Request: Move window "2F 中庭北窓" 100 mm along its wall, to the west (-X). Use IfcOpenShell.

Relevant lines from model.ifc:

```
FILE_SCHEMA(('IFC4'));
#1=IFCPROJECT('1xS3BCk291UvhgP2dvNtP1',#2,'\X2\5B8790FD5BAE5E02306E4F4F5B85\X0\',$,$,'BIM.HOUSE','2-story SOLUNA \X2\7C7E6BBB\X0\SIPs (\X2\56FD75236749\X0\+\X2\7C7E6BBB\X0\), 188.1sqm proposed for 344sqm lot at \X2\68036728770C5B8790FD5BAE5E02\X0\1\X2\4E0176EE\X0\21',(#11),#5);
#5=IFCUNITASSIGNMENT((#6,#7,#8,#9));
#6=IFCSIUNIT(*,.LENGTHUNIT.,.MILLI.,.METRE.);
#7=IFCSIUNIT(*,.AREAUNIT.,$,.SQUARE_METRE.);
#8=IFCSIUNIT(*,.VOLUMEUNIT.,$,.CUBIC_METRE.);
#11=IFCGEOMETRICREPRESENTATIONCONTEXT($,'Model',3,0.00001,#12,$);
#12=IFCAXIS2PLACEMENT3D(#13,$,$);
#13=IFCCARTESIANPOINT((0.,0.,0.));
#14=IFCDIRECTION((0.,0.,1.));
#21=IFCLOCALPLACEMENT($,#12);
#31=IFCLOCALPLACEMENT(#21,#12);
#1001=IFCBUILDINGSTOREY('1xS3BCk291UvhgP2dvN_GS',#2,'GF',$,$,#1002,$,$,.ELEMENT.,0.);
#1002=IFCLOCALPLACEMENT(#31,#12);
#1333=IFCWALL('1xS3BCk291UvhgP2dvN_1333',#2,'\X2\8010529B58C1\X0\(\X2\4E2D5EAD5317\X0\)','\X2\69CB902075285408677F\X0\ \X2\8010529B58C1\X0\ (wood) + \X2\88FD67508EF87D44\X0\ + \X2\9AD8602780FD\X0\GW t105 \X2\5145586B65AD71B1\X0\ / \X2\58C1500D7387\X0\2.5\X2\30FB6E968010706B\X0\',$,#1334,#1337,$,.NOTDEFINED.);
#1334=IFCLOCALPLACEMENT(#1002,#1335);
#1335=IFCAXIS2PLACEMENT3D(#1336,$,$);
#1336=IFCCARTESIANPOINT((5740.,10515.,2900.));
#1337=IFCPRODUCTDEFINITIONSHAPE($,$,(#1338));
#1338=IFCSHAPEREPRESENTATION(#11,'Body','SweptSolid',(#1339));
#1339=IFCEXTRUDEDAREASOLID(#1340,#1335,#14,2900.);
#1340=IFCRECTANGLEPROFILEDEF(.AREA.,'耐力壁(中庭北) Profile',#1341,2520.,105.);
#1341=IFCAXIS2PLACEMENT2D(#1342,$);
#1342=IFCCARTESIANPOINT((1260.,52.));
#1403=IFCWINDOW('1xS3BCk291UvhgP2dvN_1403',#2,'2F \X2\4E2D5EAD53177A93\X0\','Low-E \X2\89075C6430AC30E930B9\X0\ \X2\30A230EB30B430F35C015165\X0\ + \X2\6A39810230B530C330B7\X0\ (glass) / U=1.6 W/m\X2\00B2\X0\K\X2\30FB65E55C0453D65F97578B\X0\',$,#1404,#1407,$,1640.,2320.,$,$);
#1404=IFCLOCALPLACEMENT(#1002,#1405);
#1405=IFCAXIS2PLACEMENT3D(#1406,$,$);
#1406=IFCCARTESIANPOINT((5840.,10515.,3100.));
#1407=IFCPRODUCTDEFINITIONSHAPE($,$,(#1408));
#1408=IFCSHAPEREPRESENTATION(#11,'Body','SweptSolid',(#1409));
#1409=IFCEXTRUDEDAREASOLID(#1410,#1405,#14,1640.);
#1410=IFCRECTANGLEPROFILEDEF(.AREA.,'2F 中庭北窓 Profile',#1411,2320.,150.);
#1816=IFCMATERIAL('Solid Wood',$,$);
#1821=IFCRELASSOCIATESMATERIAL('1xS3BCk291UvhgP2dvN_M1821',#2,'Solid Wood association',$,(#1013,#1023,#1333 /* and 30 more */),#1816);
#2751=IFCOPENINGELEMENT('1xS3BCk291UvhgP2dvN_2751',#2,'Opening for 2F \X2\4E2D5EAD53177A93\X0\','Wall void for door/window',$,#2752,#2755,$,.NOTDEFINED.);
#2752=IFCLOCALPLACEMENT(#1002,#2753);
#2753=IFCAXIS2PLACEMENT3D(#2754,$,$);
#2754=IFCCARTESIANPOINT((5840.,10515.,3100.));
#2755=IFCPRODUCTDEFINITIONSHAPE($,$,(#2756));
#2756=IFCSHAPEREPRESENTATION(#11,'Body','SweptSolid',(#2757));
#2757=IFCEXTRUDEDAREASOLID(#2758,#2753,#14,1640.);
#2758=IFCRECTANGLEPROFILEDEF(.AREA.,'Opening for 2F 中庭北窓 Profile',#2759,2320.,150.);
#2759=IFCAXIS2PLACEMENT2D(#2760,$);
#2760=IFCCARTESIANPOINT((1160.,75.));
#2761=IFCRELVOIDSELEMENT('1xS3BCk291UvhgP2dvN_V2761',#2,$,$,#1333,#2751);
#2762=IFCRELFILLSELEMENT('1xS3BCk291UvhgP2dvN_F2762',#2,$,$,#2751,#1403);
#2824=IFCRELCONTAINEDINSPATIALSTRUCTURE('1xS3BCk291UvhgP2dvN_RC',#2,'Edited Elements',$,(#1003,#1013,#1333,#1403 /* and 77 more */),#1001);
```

```python
import ifcopenshell
import ifcopenshell.api.geometry
import ifcopenshell.util.placement
import ifcopenshell.util.unit

model = ifcopenshell.open("model.ifc")
unit_scale = ifcopenshell.util.unit.calculate_unit_scale(model)

window = model.by_id(1403)
opening = window.FillsVoids[0].RelatingOpeningElement
wall = opening.VoidsElements[0].RelatingBuildingElement

wall_matrix = ifcopenshell.util.placement.get_local_placement(wall.ObjectPlacement)
shift = wall_matrix[:3, 0] * -0.1 / unit_scale
before = ifcopenshell.util.placement.get_local_placement(window.ObjectPlacement)[:3, 3].copy()

# The window is not placed relative to its opening, so move both.
for product in (opening, window):
    matrix = ifcopenshell.util.placement.get_local_placement(product.ObjectPlacement)
    matrix[:3, 3] += shift
    ifcopenshell.api.geometry.edit_object_placement(model, product=product, matrix=matrix, is_si=False)

after = ifcopenshell.util.placement.get_local_placement(window.ObjectPlacement)[:3, 3]
print("window moved by", (after - before).round(3) + 0.0)

model.write("model_edited.ifc")
```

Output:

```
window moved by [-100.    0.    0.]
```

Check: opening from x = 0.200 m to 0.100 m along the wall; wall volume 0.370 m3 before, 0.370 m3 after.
